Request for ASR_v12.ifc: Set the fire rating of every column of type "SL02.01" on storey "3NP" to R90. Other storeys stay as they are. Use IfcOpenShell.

First a look at what the model holds.

```python
import ifcopenshell
import ifcopenshell.util.element

model = ifcopenshell.open("ASR_v12.ifc")
print(model.schema)
storey = next(s for s in model.by_type("IfcBuildingStorey") if s.Name == "3NP")
columns = [e for e in ifcopenshell.util.element.get_decomposition(storey) if e.is_a("IfcColumn")]
seen = {}
for e in columns:
    element_type = ifcopenshell.util.element.get_type(e)
    key = (element_type.Name if element_type != e and element_type else None, ifcopenshell.util.element.get_pset(e, "Pset_ColumnCommon", "FireRating"))
    seen[key] = seen.get(key, 0) + 1
for (name, value), count in sorted(seen.items(), key=str):
    print(count, "x", name, "|", value)
```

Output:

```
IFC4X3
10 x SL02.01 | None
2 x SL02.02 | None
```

```python
import ifcopenshell
import ifcopenshell.api.pset
import ifcopenshell.util.element

model = ifcopenshell.open("ASR_v12.ifc")

storey = next(s for s in model.by_type("IfcBuildingStorey") if s.Name == "3NP")
columns = [e for e in ifcopenshell.util.element.get_decomposition(storey) if e.is_a("IfcColumn")]

count = 0
for e in columns:
    element_type = ifcopenshell.util.element.get_type(e)
    if element_type in (None, e) or element_type.Name != "SL02.01":
        continue
    # add_pset returns the element's existing set when there is one.
    pset = ifcopenshell.api.pset.add_pset(model, product=e, name="Pset_ColumnCommon")
    ifcopenshell.api.pset.edit_pset(model, pset=pset, properties={"FireRating": "R90"})
    count += 1

print(count, "columns updated")

model.write("ASR_v12_edited.ifc")
```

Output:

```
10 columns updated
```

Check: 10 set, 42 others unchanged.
